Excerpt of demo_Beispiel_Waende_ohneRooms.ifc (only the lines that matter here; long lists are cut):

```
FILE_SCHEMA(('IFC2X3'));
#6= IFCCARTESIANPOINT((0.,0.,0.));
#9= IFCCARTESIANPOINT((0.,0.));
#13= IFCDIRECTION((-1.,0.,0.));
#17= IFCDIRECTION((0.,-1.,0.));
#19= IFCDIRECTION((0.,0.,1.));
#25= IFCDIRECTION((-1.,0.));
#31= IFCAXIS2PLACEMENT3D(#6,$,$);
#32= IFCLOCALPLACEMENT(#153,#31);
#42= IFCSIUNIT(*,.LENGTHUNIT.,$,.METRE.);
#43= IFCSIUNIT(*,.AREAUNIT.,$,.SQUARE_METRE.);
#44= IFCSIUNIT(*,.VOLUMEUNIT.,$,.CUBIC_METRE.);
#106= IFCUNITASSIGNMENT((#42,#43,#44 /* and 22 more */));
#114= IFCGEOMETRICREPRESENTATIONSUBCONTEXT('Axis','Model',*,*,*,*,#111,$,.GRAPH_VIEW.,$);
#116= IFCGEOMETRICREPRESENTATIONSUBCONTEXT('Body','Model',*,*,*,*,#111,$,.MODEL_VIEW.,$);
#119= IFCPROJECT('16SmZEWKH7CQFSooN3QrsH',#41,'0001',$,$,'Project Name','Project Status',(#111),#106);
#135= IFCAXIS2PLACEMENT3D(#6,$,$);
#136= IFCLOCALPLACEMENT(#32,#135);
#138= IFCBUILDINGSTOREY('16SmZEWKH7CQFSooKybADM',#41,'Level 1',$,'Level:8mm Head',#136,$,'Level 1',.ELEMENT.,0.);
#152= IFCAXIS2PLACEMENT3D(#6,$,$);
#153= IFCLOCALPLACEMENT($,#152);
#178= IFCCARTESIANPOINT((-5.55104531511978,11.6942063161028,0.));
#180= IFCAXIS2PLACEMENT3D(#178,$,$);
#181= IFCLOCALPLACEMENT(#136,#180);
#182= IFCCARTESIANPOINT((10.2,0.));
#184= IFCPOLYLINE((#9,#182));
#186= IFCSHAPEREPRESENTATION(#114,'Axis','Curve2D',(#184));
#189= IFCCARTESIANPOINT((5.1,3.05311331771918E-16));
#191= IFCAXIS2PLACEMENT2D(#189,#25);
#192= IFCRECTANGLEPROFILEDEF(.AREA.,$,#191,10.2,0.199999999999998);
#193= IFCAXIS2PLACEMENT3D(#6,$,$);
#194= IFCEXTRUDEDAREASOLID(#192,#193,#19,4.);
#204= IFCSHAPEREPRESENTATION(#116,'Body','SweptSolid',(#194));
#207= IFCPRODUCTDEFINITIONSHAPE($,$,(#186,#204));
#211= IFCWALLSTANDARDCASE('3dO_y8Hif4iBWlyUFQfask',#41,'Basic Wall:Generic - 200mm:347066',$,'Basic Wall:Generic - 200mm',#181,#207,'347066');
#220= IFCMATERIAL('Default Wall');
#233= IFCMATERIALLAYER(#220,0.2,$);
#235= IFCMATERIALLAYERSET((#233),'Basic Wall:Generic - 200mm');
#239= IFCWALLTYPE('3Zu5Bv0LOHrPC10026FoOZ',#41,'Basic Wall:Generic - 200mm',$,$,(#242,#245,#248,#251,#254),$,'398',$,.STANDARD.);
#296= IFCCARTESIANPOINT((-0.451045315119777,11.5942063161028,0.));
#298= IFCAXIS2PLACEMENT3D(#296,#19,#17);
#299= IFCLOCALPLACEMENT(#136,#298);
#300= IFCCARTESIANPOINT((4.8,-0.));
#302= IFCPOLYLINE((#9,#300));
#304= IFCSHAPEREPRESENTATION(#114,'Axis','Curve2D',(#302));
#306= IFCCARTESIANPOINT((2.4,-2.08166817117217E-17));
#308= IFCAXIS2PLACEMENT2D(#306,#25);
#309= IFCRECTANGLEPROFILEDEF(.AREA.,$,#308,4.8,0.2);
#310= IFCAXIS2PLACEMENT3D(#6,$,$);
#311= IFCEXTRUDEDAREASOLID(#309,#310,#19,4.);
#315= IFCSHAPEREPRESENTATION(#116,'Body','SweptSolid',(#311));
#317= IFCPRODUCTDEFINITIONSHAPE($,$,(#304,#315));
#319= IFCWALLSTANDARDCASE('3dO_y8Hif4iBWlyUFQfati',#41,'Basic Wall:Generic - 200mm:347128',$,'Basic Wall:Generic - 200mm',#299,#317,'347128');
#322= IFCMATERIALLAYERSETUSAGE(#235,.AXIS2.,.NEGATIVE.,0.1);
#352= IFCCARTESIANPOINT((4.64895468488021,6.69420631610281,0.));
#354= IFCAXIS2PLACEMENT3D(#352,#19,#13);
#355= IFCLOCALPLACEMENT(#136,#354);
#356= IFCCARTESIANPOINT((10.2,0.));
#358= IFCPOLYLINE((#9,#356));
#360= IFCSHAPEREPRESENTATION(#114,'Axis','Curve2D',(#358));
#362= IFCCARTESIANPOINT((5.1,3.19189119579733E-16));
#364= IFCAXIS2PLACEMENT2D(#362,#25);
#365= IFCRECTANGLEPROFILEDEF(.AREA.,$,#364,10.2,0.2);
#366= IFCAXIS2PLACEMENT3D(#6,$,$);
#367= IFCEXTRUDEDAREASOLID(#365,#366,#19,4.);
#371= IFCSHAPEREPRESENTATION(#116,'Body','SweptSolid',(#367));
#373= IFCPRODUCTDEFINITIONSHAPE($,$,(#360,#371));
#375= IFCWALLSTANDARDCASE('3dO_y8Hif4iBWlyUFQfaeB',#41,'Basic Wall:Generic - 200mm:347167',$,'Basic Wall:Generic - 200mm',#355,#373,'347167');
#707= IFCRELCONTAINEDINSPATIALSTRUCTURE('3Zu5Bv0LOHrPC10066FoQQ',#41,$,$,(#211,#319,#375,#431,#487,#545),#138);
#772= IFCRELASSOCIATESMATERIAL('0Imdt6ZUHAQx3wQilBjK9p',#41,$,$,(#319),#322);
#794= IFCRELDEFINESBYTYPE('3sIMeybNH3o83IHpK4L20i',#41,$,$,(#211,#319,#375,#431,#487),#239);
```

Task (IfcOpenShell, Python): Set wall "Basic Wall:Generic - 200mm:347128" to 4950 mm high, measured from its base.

```python
import ifcopenshell
import ifcopenshell.geom
import ifcopenshell.util.representation
import ifcopenshell.util.shape

model = ifcopenshell.open("demo_Beispiel_Waende_ohneRooms.ifc")
settings = ifcopenshell.geom.settings()


def volume(element):
    """Net volume in cubic metres, openings subtracted."""
    shape = ifcopenshell.geom.create_shape(settings, element)
    return ifcopenshell.util.shape.get_volume(shape.geometry)


wall = model.by_guid("3dO_y8Hif4iBWlyUFQfati")
before = volume(wall)

body = ifcopenshell.util.representation.get_representation(wall, "Model", "Body")
solid = body.Items[0]
old_height = solid.Depth
solid.Depth = 4.95
after = volume(wall)

print(f"height {old_height:g} -> {solid.Depth:g}, volume {before:.3f} -> {after:.3f} m3")

model.write("demo_Beispiel_Waende_ohneRooms_rev.ifc")
```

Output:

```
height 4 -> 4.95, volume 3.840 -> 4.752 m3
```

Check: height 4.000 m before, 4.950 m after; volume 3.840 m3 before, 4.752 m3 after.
